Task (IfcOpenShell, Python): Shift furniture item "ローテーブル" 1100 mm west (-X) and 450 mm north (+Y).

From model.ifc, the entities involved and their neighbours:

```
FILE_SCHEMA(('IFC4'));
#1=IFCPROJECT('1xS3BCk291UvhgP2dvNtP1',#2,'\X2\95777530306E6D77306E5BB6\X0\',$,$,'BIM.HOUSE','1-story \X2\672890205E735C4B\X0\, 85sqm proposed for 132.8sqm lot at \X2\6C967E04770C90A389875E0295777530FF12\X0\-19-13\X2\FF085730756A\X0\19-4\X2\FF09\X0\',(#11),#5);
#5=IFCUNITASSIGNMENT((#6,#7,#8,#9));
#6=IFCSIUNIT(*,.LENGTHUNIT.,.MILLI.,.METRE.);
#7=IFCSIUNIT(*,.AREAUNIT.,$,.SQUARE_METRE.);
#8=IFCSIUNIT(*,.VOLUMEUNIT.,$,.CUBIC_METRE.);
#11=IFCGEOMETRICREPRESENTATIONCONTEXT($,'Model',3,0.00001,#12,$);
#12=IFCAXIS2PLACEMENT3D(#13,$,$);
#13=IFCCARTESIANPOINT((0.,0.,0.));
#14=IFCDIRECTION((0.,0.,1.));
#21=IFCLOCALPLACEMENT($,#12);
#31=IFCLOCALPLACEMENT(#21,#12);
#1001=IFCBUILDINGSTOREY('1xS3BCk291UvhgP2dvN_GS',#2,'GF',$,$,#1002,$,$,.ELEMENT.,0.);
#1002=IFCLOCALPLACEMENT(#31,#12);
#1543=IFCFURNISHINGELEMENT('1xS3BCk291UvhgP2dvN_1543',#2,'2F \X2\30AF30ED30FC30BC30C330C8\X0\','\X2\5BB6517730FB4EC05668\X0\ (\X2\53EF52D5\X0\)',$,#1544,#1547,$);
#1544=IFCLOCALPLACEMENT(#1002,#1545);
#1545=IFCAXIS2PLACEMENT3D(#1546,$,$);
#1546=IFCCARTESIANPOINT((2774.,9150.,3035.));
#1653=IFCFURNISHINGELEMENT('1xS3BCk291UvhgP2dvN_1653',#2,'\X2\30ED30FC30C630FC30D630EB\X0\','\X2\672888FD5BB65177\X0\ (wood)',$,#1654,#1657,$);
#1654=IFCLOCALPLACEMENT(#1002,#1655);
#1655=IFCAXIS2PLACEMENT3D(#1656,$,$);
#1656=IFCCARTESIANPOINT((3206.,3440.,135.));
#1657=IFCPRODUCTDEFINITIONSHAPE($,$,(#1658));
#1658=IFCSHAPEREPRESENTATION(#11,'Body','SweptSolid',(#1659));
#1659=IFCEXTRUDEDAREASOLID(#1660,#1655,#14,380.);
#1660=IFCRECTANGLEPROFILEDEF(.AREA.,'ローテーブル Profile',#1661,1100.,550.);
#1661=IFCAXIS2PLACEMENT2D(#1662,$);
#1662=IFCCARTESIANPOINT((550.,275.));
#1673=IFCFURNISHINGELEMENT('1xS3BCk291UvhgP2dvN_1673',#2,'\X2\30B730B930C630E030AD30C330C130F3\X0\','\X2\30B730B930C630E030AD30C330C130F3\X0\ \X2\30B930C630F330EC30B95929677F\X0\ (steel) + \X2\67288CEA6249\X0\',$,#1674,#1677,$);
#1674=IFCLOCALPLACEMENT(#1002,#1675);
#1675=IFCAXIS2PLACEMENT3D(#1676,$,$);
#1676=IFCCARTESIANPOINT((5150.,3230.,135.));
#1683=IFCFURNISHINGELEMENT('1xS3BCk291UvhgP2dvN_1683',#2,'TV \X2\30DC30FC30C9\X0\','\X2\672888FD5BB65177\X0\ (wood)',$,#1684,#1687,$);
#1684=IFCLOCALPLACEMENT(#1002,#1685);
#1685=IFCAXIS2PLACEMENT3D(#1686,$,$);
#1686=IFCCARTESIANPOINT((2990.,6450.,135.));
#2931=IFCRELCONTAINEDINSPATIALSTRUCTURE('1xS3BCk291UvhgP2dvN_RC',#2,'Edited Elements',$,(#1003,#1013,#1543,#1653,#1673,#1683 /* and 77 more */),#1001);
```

```python
import ifcopenshell
import ifcopenshell.api.geometry
import ifcopenshell.util.placement
import ifcopenshell.util.unit

model = ifcopenshell.open("model.ifc")
unit_scale = ifcopenshell.util.unit.calculate_unit_scale(model)

item = model.by_guid("1xS3BCk291UvhgP2dvN_1653")
matrix = ifcopenshell.util.placement.get_local_placement(item.ObjectPlacement)
matrix[0, 3] -= 1.1 / unit_scale
matrix[1, 3] += 0.45 / unit_scale
ifcopenshell.api.geometry.edit_object_placement(model, product=item, matrix=matrix, is_si=False)

print(ifcopenshell.util.placement.get_local_placement(item.ObjectPlacement).round(3) + 0.0)

model.write("model_rev.ifc")
```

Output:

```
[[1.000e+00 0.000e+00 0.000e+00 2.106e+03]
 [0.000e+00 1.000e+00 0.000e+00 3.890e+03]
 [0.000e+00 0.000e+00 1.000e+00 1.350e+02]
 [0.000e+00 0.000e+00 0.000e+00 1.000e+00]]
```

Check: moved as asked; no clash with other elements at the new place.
